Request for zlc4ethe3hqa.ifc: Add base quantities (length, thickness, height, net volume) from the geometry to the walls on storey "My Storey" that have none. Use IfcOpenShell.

First a look at what the model holds.

```python
import ifcopenshell
import ifcopenshell.util.element
import ifcopenshell.util.unit

model = ifcopenshell.open("zlc4ethe3hqa.ifc")
print(model.schema)
for unit_type in ("LENGTHUNIT", "AREAUNIT", "VOLUMEUNIT"):
    print(unit_type, ifcopenshell.util.unit.calculate_unit_scale(model, unit_type))
storey = next(s for s in model.by_type("IfcBuildingStorey") if s.Name == "My Storey")
walls = [e for e in ifcopenshell.util.element.get_decomposition(storey) if e.is_a("IfcWall")]
for e in sorted(walls, key=lambda e: e.id()):
    print(e.id(), e.is_a(), e.Name, list(ifcopenshell.util.element.get_psets(e, qtos_only=True)), sep=" | ")
```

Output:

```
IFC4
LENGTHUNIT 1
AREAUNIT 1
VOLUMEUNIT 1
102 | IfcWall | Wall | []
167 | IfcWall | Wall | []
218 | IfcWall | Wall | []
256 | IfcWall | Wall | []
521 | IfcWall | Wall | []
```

```python
import ifcopenshell
import ifcopenshell.api.pset
import ifcopenshell.geom
import ifcopenshell.util.element
import ifcopenshell.util.shape
import ifcopenshell.util.unit

model = ifcopenshell.open("zlc4ethe3hqa.ifc")
unit_scale = ifcopenshell.util.unit.calculate_unit_scale(model)
volume_scale = ifcopenshell.util.unit.calculate_unit_scale(model, "VOLUMEUNIT")
settings = ifcopenshell.geom.settings()

storey = next(s for s in model.by_type("IfcBuildingStorey") if s.Name == "My Storey")
walls = [e for e in ifcopenshell.util.element.get_decomposition(storey) if e.is_a("IfcWall")]

for e in sorted(walls, key=lambda e: e.id()):
    if ifcopenshell.util.element.get_psets(e, qtos_only=True, should_inherit=False):
        continue
    # Geometry comes back in metres, in the element's own axes.
    shape = ifcopenshell.geom.create_shape(settings, e)
    values = {
        "Length": ifcopenshell.util.shape.get_x(shape.geometry) / unit_scale,
        "Width": ifcopenshell.util.shape.get_y(shape.geometry) / unit_scale,
        "Height": ifcopenshell.util.shape.get_z(shape.geometry) / unit_scale,
        "NetVolume": ifcopenshell.util.shape.get_volume(shape.geometry) / volume_scale,
    }
    qto = ifcopenshell.api.pset.add_qto(model, product=e, name="Qto_WallBaseQuantities")
    ifcopenshell.api.pset.edit_qto(model, qto=qto, properties=values)
    print(e.id(), {k: round(v, 3) for k, v in values.items()})

model.write("zlc4ethe3hqa_v2.ifc")
```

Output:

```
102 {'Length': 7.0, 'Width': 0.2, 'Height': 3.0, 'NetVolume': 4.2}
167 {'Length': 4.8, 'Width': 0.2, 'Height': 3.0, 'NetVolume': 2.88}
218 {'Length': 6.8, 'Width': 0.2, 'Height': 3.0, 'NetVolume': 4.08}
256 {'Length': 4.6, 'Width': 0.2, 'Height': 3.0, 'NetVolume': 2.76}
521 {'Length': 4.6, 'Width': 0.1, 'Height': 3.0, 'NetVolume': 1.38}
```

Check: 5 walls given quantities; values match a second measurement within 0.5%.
